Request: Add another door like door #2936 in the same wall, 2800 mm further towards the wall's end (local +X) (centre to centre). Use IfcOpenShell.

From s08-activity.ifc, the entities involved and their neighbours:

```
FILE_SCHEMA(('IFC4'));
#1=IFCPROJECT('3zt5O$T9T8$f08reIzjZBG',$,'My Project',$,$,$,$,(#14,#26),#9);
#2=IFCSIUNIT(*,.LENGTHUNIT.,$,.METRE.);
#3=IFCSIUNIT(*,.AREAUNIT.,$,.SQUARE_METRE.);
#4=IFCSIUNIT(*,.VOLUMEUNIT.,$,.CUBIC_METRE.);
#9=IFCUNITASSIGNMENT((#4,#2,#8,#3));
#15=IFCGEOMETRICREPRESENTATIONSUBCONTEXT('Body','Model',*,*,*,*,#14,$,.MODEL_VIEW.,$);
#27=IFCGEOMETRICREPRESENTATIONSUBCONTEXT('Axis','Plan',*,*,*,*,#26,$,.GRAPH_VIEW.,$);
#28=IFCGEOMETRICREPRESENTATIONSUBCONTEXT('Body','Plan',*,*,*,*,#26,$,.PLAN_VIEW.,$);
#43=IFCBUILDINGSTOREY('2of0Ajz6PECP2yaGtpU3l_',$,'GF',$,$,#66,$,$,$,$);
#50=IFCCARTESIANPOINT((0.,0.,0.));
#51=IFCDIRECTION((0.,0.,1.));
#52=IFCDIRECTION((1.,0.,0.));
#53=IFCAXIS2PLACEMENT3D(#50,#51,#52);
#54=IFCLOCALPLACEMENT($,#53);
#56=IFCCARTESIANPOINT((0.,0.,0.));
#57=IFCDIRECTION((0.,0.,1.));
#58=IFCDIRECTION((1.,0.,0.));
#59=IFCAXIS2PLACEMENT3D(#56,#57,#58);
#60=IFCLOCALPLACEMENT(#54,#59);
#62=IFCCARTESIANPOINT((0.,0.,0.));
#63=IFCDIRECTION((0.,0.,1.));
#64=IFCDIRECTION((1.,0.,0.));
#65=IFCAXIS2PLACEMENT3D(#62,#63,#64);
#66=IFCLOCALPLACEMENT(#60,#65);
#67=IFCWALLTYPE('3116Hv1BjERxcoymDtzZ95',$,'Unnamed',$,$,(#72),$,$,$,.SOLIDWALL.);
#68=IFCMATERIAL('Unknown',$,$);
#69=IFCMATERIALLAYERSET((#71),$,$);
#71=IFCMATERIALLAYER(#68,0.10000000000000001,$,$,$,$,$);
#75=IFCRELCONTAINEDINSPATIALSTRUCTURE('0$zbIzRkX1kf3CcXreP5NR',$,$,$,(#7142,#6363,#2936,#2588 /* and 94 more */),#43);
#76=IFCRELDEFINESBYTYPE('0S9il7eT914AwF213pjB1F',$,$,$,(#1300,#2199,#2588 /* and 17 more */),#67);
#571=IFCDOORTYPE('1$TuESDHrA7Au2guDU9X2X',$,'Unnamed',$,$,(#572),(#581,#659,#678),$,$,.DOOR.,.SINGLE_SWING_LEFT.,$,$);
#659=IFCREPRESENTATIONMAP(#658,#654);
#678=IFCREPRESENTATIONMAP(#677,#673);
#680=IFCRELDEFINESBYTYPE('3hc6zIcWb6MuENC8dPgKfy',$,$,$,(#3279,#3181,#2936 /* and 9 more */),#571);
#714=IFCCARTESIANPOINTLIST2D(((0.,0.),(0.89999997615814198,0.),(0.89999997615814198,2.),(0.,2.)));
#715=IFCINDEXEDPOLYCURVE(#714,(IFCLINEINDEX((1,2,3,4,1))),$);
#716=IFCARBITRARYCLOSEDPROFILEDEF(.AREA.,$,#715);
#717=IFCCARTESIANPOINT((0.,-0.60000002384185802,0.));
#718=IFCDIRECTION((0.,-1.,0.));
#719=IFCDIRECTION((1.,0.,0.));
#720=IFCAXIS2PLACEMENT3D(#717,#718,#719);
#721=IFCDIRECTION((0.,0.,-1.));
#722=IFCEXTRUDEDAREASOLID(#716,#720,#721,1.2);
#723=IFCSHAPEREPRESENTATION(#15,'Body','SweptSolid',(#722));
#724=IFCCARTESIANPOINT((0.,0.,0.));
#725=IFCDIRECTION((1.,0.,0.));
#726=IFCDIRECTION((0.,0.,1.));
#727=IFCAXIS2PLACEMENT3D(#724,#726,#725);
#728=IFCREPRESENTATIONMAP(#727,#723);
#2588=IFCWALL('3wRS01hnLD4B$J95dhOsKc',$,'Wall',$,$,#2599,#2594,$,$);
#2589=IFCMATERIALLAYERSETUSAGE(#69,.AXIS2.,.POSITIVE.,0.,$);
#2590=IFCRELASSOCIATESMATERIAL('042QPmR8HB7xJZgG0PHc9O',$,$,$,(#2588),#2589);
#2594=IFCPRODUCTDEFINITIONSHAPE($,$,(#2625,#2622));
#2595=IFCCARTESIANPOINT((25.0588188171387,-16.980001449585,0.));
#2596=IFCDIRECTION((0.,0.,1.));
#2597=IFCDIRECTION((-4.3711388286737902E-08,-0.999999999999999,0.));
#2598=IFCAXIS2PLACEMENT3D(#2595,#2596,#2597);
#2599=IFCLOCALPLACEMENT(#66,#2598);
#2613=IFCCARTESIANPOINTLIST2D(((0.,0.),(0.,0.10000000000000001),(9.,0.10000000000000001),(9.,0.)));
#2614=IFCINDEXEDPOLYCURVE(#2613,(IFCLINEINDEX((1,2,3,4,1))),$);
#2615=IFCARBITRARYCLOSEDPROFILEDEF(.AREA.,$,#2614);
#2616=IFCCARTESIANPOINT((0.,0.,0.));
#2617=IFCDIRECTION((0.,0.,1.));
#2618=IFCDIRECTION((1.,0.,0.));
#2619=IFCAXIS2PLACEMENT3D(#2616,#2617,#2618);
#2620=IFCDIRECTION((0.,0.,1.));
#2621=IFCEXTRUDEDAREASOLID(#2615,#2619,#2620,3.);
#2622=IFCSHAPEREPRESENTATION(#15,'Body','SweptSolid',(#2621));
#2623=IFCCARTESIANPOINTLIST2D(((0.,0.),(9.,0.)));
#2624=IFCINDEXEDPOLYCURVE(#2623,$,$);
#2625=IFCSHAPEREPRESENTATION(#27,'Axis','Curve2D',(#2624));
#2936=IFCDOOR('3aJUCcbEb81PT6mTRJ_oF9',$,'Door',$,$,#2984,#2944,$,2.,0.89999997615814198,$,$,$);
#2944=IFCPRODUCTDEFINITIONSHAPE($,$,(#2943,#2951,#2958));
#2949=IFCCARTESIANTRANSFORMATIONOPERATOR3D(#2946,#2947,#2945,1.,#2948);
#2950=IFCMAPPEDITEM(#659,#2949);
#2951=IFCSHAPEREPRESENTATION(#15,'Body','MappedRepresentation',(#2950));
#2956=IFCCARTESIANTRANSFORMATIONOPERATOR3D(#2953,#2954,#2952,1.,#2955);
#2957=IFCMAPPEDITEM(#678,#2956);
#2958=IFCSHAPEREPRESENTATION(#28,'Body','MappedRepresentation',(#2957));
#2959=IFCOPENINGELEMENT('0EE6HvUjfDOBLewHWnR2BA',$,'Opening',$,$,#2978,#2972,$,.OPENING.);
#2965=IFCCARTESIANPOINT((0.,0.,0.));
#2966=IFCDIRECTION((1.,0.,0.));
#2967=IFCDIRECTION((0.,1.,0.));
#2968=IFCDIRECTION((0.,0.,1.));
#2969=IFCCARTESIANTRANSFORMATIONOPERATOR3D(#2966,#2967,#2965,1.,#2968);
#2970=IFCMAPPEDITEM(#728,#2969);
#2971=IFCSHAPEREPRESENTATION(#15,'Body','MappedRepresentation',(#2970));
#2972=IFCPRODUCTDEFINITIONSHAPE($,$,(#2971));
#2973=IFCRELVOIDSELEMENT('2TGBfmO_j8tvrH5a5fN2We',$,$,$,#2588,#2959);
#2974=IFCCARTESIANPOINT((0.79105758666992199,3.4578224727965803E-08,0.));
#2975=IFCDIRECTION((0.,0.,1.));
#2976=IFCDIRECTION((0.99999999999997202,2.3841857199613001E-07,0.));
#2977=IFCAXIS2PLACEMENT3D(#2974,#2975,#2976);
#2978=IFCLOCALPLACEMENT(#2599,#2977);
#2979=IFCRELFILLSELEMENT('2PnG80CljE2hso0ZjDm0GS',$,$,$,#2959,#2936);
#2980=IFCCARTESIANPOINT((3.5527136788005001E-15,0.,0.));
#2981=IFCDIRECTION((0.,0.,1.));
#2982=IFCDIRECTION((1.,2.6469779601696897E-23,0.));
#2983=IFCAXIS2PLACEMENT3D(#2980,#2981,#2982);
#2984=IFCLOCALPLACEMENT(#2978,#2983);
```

```python
import ifcopenshell
import ifcopenshell.api.feature
import ifcopenshell.api.geometry
import ifcopenshell.api.root
import ifcopenshell.geom
import ifcopenshell.util.element
import ifcopenshell.util.placement
import ifcopenshell.util.shape

model = ifcopenshell.open("s08-activity.ifc")
settings = ifcopenshell.geom.settings()


def volume(element):
    """Net volume in cubic metres, openings subtracted."""
    shape = ifcopenshell.geom.create_shape(settings, element)
    return ifcopenshell.util.shape.get_volume(shape.geometry)


door = model.by_guid("3aJUCcbEb81PT6mTRJ_oF9")
opening = door.FillsVoids[0].RelatingOpeningElement
wall = opening.VoidsElements[0].RelatingBuildingElement
before = volume(wall)
shift = ifcopenshell.util.placement.get_local_placement(wall.ObjectPlacement)[:3, 0] * 2.8

# copy_class copies the void relationship, type, container and properties, but no geometry.
new_opening = ifcopenshell.api.root.copy_class(model, product=opening)
new_opening.Representation = ifcopenshell.util.element.copy_deep(
    model, opening.Representation, exclude=["IfcGeometricRepresentationContext", "IfcRepresentationMap"]
)
new_door = ifcopenshell.api.root.copy_class(model, product=door)
new_door.Representation = ifcopenshell.util.element.copy_deep(
    model, door.Representation, exclude=["IfcGeometricRepresentationContext", "IfcRepresentationMap"]
)
ifcopenshell.api.feature.add_filling(model, opening=new_opening, element=new_door)

for old, new in ((opening, new_opening), (door, new_door)):
    matrix = ifcopenshell.util.placement.get_local_placement(old.ObjectPlacement)
    matrix[:3, 3] += shift
    ifcopenshell.api.geometry.edit_object_placement(model, product=new, matrix=matrix, is_si=False)

after = volume(wall)

print(f"wall volume {before:.3f} -> {after:.3f} m3")

model.write("s08-activity_rev.ifc")
```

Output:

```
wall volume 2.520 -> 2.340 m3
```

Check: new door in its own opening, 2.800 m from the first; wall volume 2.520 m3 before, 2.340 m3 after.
